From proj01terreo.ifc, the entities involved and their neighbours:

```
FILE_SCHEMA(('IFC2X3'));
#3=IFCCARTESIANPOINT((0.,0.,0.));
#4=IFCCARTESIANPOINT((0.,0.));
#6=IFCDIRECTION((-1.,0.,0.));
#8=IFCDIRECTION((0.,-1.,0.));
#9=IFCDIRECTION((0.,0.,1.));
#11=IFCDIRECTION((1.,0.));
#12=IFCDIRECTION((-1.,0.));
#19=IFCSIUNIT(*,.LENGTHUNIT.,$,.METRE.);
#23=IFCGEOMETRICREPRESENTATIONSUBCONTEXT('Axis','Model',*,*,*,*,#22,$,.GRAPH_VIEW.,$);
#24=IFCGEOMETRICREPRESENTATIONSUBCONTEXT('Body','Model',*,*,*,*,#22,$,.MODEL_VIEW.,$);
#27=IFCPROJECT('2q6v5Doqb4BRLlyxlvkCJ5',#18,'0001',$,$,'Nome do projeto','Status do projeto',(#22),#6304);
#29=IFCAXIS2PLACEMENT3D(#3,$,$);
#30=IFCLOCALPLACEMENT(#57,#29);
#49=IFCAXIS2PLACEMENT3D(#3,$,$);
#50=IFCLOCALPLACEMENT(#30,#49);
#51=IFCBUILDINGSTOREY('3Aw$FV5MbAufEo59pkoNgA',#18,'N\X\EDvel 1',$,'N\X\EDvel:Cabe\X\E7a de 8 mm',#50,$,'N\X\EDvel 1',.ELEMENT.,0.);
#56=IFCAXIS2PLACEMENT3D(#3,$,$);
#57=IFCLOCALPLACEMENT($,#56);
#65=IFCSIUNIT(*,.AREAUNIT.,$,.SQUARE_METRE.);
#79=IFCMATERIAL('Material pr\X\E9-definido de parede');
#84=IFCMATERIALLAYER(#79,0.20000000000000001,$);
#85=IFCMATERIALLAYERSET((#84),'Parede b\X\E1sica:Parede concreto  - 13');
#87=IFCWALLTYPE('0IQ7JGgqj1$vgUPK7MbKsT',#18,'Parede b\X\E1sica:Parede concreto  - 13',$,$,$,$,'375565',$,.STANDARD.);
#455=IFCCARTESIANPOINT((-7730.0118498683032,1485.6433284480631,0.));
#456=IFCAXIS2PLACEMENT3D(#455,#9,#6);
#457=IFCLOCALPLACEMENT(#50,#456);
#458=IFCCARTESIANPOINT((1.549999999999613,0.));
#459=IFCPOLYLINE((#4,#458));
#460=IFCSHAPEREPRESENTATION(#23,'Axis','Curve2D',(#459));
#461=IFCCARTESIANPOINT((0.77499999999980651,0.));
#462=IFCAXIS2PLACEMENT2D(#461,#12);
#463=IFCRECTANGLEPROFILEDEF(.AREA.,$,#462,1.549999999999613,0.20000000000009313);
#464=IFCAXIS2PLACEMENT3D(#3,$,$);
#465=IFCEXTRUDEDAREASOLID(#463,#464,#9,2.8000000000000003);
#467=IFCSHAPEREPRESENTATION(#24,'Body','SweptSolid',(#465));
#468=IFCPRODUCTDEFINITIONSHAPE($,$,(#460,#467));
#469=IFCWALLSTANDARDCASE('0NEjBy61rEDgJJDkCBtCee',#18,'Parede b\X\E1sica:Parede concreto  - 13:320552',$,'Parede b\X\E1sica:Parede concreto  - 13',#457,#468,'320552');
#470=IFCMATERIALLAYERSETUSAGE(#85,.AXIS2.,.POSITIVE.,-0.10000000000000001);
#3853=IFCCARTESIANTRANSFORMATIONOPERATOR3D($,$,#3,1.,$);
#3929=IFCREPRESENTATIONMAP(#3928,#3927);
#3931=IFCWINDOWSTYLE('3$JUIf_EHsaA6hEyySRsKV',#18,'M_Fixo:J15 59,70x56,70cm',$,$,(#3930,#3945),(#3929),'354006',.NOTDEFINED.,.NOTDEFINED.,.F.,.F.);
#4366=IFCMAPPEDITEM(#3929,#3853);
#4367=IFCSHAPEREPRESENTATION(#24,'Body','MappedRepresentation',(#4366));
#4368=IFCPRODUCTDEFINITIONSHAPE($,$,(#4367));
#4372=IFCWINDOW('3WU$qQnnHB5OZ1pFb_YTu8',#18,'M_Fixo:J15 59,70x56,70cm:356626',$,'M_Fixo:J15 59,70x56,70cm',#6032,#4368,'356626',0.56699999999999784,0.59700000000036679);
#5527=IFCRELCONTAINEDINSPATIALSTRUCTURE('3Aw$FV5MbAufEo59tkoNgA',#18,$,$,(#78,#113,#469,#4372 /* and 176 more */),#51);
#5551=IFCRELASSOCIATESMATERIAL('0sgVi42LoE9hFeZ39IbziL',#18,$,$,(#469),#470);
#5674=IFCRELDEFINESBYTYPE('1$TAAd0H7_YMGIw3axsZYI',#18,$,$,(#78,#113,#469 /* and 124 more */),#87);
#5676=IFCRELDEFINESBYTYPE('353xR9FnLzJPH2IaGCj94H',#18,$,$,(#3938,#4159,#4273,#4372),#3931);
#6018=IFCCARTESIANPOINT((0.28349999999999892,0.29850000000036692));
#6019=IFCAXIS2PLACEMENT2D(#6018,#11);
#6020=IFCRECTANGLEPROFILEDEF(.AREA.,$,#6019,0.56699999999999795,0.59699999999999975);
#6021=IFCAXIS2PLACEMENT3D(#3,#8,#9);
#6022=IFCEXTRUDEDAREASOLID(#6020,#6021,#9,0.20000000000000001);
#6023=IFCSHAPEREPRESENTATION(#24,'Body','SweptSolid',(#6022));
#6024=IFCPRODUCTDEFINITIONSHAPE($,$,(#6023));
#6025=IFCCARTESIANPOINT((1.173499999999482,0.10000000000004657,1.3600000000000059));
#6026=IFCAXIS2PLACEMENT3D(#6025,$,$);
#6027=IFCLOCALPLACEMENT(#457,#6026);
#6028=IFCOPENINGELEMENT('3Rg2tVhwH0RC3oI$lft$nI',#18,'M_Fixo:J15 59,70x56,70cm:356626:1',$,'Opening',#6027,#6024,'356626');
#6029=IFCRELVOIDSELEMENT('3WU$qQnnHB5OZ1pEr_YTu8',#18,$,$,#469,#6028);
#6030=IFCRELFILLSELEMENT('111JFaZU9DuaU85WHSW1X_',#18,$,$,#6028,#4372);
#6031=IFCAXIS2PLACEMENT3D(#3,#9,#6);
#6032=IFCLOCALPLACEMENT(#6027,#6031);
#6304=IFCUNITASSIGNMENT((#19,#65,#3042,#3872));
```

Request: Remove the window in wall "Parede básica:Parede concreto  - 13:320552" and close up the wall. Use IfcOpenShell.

```python
import ifcopenshell
import ifcopenshell.api.feature
import ifcopenshell.api.root
import ifcopenshell.geom
import ifcopenshell.util.shape

model = ifcopenshell.open("proj01terreo.ifc")
settings = ifcopenshell.geom.settings()


def volume(element):
    """Net volume in cubic metres, openings subtracted."""
    shape = ifcopenshell.geom.create_shape(settings, element)
    return ifcopenshell.util.shape.get_volume(shape.geometry)


window = model.by_id(4372)
opening = window.FillsVoids[0].RelatingOpeningElement
wall = opening.VoidsElements[0].RelatingBuildingElement
before = volume(wall)

ifcopenshell.api.root.remove_product(model, product=window)
ifcopenshell.api.feature.remove_feature(model, feature=opening)

after = volume(wall)

print(f"wall volume {before:.3f} -> {after:.3f} m3")

model.write("proj01terreo_rev.ifc")
```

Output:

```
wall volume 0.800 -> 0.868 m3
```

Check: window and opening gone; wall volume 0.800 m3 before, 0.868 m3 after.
